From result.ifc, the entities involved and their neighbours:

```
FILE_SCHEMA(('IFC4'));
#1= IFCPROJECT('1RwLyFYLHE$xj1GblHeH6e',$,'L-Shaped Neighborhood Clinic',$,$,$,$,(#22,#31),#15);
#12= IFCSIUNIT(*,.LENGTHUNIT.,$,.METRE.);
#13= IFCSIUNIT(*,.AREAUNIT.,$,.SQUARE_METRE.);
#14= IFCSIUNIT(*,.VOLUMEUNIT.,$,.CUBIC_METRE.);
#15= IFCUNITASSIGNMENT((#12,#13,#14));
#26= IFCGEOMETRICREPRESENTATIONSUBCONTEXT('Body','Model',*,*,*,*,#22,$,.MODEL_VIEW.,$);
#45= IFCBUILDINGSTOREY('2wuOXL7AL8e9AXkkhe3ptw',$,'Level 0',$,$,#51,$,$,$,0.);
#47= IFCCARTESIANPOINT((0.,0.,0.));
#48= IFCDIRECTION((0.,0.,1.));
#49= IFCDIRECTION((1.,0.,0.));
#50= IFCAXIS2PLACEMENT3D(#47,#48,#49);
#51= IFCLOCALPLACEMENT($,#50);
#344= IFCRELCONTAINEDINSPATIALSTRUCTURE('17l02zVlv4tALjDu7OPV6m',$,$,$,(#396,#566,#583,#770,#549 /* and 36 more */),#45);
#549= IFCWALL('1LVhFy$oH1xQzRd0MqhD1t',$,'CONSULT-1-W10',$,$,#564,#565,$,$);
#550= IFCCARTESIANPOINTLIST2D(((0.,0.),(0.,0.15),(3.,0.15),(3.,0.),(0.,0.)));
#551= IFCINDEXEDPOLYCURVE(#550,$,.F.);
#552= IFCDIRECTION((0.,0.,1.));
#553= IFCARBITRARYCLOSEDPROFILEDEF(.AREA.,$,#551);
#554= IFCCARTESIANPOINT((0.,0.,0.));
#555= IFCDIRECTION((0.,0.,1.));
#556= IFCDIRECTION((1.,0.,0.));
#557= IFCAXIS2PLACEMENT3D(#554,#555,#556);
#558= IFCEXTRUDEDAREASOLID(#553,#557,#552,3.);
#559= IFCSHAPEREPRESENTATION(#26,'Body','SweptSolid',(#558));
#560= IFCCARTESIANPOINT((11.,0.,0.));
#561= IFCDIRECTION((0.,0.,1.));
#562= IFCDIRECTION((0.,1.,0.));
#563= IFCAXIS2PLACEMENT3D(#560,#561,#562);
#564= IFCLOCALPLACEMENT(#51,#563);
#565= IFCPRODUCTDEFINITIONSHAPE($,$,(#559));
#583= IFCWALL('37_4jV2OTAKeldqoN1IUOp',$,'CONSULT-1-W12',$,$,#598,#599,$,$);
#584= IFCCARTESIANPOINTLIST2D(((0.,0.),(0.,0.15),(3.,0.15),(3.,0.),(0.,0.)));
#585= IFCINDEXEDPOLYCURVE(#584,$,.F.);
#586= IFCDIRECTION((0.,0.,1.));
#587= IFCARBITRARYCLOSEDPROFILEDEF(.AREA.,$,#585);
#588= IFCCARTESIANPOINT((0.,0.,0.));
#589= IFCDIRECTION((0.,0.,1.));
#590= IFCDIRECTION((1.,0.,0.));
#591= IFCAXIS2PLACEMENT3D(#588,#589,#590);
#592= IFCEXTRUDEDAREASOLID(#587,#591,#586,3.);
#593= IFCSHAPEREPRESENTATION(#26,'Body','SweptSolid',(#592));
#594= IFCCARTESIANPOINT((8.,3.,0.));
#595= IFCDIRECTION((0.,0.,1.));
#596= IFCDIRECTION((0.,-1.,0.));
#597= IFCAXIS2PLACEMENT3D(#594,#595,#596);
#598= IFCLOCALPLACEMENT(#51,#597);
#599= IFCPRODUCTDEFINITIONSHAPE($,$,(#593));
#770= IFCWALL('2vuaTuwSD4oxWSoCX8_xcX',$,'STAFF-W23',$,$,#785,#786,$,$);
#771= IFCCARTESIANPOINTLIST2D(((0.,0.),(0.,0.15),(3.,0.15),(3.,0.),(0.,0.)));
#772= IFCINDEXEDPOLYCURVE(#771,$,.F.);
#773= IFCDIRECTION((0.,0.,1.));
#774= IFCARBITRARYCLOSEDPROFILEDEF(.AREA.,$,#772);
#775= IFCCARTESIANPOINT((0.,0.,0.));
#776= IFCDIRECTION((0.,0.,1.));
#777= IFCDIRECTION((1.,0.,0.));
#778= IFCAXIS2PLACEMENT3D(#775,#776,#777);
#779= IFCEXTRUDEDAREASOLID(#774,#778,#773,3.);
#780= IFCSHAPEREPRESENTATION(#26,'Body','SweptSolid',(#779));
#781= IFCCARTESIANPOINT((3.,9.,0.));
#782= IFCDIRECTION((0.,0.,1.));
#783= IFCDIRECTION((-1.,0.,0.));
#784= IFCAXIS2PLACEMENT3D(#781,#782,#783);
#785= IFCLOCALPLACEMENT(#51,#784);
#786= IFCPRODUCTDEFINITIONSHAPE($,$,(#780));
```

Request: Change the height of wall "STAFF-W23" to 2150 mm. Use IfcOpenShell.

```python
import ifcopenshell
import ifcopenshell.geom
import ifcopenshell.util.representation
import ifcopenshell.util.shape
import ifcopenshell.util.unit

model = ifcopenshell.open("result.ifc")
unit_scale = ifcopenshell.util.unit.calculate_unit_scale(model)
settings = ifcopenshell.geom.settings()


def volume(element):
    """Net volume in cubic metres, openings subtracted."""
    shape = ifcopenshell.geom.create_shape(settings, element)
    return ifcopenshell.util.shape.get_volume(shape.geometry)


wall = model.by_guid("2vuaTuwSD4oxWSoCX8_xcX")
before = volume(wall)

body = ifcopenshell.util.representation.get_representation(wall, "Model", "Body")
solid = body.Items[0]
old_height = solid.Depth
solid.Depth = 2.15 / unit_scale
after = volume(wall)

print(f"height {old_height:g} -> {solid.Depth:g}, volume {before:.3f} -> {after:.3f} m3")

model.write("result-out.ifc")
```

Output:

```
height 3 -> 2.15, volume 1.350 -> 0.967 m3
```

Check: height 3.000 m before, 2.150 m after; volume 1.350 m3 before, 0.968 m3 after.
